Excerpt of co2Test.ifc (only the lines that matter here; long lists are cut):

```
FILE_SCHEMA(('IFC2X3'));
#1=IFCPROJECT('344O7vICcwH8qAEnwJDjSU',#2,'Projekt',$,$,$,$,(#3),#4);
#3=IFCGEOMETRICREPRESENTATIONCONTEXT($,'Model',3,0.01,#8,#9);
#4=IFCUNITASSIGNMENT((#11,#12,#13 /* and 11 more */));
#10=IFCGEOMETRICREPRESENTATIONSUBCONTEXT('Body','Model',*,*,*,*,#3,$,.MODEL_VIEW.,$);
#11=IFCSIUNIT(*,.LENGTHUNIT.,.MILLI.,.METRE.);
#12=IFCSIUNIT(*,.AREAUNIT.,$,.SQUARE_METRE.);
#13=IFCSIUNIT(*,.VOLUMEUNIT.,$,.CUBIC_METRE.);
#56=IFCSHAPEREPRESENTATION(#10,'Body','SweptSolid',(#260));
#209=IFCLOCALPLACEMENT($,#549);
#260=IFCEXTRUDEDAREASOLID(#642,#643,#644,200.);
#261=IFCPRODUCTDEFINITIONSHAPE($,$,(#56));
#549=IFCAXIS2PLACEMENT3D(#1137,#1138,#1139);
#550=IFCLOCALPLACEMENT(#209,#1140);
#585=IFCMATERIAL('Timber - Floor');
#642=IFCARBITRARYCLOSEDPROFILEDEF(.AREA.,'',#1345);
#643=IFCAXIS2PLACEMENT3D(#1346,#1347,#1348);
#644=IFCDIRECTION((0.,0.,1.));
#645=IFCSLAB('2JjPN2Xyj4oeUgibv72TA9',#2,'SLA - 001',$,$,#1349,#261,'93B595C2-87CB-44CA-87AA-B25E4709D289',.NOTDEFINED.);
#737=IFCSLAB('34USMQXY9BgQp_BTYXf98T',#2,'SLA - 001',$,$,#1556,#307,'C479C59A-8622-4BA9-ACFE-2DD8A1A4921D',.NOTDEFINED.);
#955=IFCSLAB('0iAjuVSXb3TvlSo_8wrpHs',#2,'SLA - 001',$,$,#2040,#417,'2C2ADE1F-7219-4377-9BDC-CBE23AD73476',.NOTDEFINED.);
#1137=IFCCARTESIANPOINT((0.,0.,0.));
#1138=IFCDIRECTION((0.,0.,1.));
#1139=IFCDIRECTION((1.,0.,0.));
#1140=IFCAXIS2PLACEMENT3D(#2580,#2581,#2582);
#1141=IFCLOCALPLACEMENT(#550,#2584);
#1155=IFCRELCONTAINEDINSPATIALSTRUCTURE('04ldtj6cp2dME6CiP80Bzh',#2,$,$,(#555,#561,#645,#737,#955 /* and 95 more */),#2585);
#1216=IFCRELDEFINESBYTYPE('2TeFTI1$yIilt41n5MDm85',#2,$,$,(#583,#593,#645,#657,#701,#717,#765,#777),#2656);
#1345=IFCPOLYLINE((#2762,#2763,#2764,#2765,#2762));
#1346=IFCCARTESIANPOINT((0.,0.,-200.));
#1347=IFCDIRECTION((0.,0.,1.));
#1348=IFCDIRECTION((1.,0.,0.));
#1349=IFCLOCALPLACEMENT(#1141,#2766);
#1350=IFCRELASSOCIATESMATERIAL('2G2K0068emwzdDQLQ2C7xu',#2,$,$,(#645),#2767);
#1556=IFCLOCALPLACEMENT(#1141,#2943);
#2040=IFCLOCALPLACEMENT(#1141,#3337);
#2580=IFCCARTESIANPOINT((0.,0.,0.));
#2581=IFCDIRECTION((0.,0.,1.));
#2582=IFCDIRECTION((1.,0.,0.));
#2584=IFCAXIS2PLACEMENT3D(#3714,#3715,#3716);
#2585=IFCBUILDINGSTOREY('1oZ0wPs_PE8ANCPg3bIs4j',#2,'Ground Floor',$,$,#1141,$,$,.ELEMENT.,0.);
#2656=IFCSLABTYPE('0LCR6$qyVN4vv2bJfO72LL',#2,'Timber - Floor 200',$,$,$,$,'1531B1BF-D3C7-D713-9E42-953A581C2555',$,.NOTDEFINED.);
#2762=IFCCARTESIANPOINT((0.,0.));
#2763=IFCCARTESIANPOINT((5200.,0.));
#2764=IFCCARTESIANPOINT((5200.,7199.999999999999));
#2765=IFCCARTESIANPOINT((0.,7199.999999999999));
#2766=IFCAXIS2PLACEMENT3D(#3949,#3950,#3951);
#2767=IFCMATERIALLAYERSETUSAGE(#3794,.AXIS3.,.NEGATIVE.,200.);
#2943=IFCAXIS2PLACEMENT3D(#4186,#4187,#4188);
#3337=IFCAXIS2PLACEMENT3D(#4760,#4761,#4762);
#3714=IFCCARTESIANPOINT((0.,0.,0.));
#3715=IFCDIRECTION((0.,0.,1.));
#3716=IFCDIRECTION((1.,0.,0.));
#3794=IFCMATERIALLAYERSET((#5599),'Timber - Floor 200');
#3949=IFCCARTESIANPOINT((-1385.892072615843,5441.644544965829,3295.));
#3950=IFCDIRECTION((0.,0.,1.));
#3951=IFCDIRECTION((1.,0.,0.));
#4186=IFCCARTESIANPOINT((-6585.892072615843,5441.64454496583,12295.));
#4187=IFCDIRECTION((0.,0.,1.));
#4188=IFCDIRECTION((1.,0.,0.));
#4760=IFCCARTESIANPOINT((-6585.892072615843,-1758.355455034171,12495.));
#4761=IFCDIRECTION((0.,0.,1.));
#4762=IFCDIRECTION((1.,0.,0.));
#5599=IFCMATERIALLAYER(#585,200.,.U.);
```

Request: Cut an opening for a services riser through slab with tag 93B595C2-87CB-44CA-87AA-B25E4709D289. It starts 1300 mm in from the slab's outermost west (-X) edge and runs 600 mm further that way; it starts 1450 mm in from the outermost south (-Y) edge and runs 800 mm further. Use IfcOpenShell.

```python
import numpy as np
import ifcopenshell
import ifcopenshell.api.feature
import ifcopenshell.api.geometry
import ifcopenshell.api.root
import ifcopenshell.geom
import ifcopenshell.util.placement
import ifcopenshell.util.representation
import ifcopenshell.util.shape
import ifcopenshell.util.unit

model = ifcopenshell.open("co2Test.ifc")
unit_scale = ifcopenshell.util.unit.calculate_unit_scale(model)
settings = ifcopenshell.geom.settings()


def volume(element):
    """Net volume in cubic metres, openings subtracted."""
    shape = ifcopenshell.geom.create_shape(settings, element)
    return ifcopenshell.util.shape.get_volume(shape.geometry)


slab = model.by_id(645)
before = volume(slab)

# Extent in the slab's own axes, in metres. The edges named are its -X and -Y sides.
slab_shape = ifcopenshell.geom.create_shape(settings, slab)
vertices = ifcopenshell.util.shape.get_vertices(slab_shape.geometry)
x_min, y_min, bottom = vertices.min(axis=0)
top = vertices[:, 2].max()

opening = ifcopenshell.api.root.create_entity(model, ifc_class="IfcOpeningElement", name="Services riser opening")
context = ifcopenshell.util.representation.get_context(model, "Model", "Body", "MODEL_VIEW")
width, depth = 0.6, 0.8
outline = [(0.0, 0.0), (width, 0.0), (width, depth), (0.0, depth), (0.0, 0.0)]
# Overshoot both faces by 50 mm so the cut is clean.
shape = ifcopenshell.api.geometry.add_slab_representation(
    model, context=context, depth=top - bottom + 0.1, polyline=outline
)
ifcopenshell.api.geometry.assign_representation(model, product=opening, representation=shape)

matrix = ifcopenshell.util.placement.get_local_placement(slab.ObjectPlacement)
matrix[:, 3] = matrix @ np.append(np.array([x_min + 1.3, y_min + 1.45, bottom - 0.05]) / unit_scale, 1.0)
ifcopenshell.api.geometry.edit_object_placement(model, product=opening, matrix=matrix, is_si=False)
ifcopenshell.api.feature.add_feature(model, feature=opening, element=slab)

after = volume(slab)

print(f"slab volume {before:.3f} -> {after:.3f} m3")

model.write("co2Test_updated.ifc")
```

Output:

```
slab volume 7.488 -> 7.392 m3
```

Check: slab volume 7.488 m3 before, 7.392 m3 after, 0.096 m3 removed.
